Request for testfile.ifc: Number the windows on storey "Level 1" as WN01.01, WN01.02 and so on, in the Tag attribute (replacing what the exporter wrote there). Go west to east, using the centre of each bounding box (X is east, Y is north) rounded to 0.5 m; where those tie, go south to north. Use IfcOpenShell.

First a look at what the model holds.

```python
import ifcopenshell
import ifcopenshell.util.element
import ifcopenshell.util.placement

model = ifcopenshell.open("testfile.ifc")
print(model.schema)
storey = next(s for s in model.by_type("IfcBuildingStorey") if s.Name == "Level 1")
windows = [e for e in ifcopenshell.util.element.get_decomposition(storey) if e.is_a("IfcWindow")]
for e in sorted(windows, key=lambda e: e.id()):
    origin = ifcopenshell.util.placement.get_local_placement(e.ObjectPlacement)[:3, 3]
    print(e.id(), e.Tag, e.Name, origin.round(2) + 0.0, sep=" | ")
```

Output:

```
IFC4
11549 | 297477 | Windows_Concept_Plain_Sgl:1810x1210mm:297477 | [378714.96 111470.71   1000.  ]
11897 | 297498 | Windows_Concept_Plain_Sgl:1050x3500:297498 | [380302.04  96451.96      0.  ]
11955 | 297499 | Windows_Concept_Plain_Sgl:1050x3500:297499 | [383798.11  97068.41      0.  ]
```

```python
import ifcopenshell
import ifcopenshell.geom
import ifcopenshell.util.element
import ifcopenshell.util.shape

model = ifcopenshell.open("testfile.ifc")
settings = ifcopenshell.geom.settings()
settings.set("use-world-coords", True)


def centre(element):
    shape = ifcopenshell.geom.create_shape(settings, element)
    return ifcopenshell.util.shape.get_bbox_centroid(shape.geometry)


storey = next(s for s in model.by_type("IfcBuildingStorey") if s.Name == "Level 1")
windows = [e for e in ifcopenshell.util.element.get_decomposition(storey) if e.is_a("IfcWindow")]

# Insertion points can sit at a corner or the storey origin, so sort by the geometry (in metres).
centres = {e: centre(e) for e in windows}
windows.sort(key=lambda e: (round(centres[e][0] / 0.5), centres[e][1]))

for i, e in enumerate(windows, start=1):
    number = f"WN01.{i:02d}"
    e.Tag = number
    print(e.id(), number)

model.write("testfile_updated.ifc")
```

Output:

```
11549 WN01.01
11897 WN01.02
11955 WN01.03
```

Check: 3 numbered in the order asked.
